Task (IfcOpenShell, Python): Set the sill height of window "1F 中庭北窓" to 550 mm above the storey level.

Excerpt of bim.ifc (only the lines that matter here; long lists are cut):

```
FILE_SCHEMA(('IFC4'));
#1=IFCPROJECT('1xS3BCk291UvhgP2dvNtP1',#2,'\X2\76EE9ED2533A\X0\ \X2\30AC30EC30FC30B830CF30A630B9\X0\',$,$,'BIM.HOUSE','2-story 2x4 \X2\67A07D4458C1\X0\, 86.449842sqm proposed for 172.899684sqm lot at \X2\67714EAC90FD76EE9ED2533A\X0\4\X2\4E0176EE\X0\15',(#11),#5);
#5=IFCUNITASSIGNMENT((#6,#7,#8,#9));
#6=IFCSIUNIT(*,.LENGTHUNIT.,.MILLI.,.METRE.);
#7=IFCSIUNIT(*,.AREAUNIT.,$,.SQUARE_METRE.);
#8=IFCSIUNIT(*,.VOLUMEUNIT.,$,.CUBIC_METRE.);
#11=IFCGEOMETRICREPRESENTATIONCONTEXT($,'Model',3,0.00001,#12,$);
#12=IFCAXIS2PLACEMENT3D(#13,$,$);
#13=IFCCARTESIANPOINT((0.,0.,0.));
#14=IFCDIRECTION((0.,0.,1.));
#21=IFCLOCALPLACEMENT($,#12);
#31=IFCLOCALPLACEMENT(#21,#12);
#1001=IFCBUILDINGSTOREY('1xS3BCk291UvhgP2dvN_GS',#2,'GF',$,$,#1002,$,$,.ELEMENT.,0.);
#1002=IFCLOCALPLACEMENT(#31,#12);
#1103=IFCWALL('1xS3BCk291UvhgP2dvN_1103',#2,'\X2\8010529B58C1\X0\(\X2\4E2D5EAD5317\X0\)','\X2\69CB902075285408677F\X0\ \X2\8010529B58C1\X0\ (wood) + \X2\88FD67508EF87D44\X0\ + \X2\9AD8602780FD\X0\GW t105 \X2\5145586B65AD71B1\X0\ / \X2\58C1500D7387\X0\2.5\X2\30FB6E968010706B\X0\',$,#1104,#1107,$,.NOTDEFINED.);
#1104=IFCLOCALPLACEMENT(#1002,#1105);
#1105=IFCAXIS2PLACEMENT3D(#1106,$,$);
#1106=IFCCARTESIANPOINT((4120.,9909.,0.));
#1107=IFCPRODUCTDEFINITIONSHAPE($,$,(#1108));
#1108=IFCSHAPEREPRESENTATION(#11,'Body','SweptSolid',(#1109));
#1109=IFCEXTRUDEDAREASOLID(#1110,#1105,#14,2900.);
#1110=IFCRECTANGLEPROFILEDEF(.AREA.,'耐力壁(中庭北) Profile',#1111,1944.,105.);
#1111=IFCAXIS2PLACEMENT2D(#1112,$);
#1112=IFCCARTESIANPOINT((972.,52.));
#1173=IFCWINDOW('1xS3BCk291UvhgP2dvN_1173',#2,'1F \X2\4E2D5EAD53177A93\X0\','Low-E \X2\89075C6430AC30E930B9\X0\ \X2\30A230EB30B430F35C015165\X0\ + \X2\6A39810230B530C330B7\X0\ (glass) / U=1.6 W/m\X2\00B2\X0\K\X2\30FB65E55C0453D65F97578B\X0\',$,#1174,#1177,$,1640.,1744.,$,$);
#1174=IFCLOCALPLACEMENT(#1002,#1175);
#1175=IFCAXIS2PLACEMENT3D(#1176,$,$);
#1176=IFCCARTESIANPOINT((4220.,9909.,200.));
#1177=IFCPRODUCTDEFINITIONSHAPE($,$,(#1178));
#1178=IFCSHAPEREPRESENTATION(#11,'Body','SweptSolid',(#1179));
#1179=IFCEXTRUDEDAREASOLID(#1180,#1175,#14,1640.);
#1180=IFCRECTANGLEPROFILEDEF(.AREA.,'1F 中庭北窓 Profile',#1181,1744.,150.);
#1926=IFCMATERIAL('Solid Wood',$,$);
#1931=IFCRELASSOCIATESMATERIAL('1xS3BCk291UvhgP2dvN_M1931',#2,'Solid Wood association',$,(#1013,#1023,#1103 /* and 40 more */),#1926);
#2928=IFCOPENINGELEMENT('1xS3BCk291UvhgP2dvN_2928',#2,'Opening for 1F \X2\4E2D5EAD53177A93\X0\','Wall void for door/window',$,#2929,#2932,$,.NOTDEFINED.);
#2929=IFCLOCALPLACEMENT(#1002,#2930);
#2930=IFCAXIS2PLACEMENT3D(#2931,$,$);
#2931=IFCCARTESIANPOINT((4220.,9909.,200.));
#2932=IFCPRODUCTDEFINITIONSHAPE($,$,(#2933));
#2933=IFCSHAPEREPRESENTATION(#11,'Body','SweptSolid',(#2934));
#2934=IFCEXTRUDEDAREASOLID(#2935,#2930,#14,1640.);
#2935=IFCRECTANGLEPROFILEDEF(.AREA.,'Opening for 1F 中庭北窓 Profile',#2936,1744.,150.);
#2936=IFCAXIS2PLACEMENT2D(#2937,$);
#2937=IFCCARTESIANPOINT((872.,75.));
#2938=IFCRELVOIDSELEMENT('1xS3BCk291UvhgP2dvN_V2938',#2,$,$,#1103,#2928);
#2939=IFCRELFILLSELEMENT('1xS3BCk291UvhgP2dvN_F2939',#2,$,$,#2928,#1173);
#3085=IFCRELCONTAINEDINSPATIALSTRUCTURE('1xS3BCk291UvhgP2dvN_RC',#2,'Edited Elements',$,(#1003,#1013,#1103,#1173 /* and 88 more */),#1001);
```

```python
import numpy as np
import ifcopenshell
import ifcopenshell.api.geometry
import ifcopenshell.geom
import ifcopenshell.util.element
import ifcopenshell.util.placement
import ifcopenshell.util.shape
import ifcopenshell.util.unit

model = ifcopenshell.open("bim.ifc")
unit_scale = ifcopenshell.util.unit.calculate_unit_scale(model)

window = model.by_guid("1xS3BCk291UvhgP2dvN_1173")
opening = window.FillsVoids[0].RelatingOpeningElement
storey = ifcopenshell.util.element.get_container(window, ifc_class="IfcBuildingStorey")
level = ifcopenshell.util.placement.get_local_placement(storey.ObjectPlacement)[2, 3]

# The opening's origin need not be at the sill, so measure its lowest point.
shape = ifcopenshell.geom.create_shape(ifcopenshell.geom.settings(), opening)
bottom = ifcopenshell.util.shape.get_shape_bottom_elevation(shape, shape.geometry) / unit_scale
dz = level + 0.55 / unit_scale - bottom

shift = np.array([0.0, 0.0, dz])
# The window is not placed relative to its opening, so move both.
for product in (opening, window):
    matrix = ifcopenshell.util.placement.get_local_placement(product.ObjectPlacement)
    matrix[:3, 3] += shift
    ifcopenshell.api.geometry.edit_object_placement(model, product=product, matrix=matrix, is_si=False)

print(f"moved by {dz * unit_scale:+.3f} m")

model.write("bim_updated.ifc")
```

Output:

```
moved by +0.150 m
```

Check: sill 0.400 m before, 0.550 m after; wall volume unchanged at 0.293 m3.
